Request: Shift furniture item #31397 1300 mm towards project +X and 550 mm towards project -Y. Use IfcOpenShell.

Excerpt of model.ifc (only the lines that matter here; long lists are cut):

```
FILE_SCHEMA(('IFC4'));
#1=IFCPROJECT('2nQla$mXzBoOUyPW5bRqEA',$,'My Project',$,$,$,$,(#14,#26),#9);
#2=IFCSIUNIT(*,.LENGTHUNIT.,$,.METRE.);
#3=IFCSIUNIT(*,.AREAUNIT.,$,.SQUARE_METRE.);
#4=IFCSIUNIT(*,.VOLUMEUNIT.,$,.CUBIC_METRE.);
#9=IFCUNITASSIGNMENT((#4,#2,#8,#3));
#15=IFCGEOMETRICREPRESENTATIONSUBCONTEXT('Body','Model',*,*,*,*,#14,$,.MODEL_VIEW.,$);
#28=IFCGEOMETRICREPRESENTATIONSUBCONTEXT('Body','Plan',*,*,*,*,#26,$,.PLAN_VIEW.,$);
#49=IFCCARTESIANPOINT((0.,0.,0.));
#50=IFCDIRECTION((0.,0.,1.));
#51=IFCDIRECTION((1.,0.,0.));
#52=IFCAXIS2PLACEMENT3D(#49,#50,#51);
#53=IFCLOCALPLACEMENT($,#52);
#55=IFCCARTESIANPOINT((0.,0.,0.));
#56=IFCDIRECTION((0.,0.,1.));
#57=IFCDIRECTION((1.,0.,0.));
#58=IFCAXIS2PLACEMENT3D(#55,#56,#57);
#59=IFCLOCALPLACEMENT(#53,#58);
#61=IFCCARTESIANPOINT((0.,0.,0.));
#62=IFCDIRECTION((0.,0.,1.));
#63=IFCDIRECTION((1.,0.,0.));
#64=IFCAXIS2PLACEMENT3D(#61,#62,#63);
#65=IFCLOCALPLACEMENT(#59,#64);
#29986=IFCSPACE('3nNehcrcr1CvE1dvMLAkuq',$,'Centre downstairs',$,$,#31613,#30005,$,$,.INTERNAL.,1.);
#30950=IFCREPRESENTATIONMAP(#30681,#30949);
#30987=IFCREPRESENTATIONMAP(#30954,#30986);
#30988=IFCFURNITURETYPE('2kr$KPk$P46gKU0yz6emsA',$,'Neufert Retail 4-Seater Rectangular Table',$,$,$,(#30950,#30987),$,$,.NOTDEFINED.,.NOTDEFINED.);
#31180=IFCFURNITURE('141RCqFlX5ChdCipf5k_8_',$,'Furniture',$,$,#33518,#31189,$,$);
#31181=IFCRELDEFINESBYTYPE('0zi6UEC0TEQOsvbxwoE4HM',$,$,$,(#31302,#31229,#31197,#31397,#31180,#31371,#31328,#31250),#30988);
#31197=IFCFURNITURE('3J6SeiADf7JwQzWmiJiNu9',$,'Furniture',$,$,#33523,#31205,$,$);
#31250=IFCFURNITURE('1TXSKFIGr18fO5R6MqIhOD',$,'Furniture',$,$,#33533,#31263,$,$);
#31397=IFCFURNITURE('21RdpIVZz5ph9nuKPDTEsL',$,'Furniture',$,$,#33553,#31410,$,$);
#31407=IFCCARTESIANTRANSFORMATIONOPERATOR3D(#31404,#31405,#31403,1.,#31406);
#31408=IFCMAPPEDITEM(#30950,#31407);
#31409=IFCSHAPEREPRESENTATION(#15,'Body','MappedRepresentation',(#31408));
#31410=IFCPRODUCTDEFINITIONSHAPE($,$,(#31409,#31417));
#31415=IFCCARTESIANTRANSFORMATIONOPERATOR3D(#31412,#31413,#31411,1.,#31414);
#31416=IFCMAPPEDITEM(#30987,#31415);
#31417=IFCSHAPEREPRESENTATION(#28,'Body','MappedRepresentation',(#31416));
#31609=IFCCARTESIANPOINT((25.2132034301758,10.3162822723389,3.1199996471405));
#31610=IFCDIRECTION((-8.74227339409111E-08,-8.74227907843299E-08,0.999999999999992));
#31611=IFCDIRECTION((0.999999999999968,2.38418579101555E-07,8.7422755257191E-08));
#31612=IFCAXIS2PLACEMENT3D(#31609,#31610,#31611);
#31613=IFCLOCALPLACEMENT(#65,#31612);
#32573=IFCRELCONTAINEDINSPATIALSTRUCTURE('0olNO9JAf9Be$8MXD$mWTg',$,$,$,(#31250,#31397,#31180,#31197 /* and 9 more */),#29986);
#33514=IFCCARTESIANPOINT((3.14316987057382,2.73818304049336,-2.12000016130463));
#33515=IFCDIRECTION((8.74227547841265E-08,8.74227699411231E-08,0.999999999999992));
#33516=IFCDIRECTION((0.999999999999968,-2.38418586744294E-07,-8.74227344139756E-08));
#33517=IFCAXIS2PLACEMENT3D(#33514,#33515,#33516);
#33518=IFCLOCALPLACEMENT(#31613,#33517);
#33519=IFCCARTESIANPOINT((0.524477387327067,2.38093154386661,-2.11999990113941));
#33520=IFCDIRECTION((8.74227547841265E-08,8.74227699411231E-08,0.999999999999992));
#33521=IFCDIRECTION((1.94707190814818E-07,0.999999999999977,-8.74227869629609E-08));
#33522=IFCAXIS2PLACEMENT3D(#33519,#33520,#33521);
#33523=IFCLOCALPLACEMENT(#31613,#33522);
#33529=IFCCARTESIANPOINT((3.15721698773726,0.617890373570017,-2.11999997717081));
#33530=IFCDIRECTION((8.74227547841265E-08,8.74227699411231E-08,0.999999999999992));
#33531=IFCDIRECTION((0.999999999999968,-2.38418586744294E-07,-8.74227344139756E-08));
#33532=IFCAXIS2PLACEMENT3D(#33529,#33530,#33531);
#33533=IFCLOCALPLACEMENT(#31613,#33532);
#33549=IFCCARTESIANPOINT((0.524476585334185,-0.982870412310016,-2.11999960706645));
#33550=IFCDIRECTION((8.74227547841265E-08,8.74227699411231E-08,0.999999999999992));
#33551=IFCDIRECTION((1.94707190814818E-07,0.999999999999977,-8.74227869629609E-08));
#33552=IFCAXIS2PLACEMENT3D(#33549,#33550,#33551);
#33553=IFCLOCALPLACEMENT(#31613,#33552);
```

```python
import ifcopenshell
import ifcopenshell.api.geometry
import ifcopenshell.util.placement
import ifcopenshell.util.unit

model = ifcopenshell.open("model.ifc")
unit_scale = ifcopenshell.util.unit.calculate_unit_scale(model)

item = model.by_guid("21RdpIVZz5ph9nuKPDTEsL")
matrix = ifcopenshell.util.placement.get_local_placement(item.ObjectPlacement)
matrix[0, 3] += 1.3 / unit_scale
matrix[1, 3] -= 0.55 / unit_scale
ifcopenshell.api.geometry.edit_object_placement(model, product=item, matrix=matrix, is_si=False)

print(ifcopenshell.util.placement.get_local_placement(item.ObjectPlacement).round(3) + 0.0)

model.write("model_updated.ifc")
```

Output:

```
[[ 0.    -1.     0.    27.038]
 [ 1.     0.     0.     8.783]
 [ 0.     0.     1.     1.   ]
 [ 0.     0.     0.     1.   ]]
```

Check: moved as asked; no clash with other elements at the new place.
